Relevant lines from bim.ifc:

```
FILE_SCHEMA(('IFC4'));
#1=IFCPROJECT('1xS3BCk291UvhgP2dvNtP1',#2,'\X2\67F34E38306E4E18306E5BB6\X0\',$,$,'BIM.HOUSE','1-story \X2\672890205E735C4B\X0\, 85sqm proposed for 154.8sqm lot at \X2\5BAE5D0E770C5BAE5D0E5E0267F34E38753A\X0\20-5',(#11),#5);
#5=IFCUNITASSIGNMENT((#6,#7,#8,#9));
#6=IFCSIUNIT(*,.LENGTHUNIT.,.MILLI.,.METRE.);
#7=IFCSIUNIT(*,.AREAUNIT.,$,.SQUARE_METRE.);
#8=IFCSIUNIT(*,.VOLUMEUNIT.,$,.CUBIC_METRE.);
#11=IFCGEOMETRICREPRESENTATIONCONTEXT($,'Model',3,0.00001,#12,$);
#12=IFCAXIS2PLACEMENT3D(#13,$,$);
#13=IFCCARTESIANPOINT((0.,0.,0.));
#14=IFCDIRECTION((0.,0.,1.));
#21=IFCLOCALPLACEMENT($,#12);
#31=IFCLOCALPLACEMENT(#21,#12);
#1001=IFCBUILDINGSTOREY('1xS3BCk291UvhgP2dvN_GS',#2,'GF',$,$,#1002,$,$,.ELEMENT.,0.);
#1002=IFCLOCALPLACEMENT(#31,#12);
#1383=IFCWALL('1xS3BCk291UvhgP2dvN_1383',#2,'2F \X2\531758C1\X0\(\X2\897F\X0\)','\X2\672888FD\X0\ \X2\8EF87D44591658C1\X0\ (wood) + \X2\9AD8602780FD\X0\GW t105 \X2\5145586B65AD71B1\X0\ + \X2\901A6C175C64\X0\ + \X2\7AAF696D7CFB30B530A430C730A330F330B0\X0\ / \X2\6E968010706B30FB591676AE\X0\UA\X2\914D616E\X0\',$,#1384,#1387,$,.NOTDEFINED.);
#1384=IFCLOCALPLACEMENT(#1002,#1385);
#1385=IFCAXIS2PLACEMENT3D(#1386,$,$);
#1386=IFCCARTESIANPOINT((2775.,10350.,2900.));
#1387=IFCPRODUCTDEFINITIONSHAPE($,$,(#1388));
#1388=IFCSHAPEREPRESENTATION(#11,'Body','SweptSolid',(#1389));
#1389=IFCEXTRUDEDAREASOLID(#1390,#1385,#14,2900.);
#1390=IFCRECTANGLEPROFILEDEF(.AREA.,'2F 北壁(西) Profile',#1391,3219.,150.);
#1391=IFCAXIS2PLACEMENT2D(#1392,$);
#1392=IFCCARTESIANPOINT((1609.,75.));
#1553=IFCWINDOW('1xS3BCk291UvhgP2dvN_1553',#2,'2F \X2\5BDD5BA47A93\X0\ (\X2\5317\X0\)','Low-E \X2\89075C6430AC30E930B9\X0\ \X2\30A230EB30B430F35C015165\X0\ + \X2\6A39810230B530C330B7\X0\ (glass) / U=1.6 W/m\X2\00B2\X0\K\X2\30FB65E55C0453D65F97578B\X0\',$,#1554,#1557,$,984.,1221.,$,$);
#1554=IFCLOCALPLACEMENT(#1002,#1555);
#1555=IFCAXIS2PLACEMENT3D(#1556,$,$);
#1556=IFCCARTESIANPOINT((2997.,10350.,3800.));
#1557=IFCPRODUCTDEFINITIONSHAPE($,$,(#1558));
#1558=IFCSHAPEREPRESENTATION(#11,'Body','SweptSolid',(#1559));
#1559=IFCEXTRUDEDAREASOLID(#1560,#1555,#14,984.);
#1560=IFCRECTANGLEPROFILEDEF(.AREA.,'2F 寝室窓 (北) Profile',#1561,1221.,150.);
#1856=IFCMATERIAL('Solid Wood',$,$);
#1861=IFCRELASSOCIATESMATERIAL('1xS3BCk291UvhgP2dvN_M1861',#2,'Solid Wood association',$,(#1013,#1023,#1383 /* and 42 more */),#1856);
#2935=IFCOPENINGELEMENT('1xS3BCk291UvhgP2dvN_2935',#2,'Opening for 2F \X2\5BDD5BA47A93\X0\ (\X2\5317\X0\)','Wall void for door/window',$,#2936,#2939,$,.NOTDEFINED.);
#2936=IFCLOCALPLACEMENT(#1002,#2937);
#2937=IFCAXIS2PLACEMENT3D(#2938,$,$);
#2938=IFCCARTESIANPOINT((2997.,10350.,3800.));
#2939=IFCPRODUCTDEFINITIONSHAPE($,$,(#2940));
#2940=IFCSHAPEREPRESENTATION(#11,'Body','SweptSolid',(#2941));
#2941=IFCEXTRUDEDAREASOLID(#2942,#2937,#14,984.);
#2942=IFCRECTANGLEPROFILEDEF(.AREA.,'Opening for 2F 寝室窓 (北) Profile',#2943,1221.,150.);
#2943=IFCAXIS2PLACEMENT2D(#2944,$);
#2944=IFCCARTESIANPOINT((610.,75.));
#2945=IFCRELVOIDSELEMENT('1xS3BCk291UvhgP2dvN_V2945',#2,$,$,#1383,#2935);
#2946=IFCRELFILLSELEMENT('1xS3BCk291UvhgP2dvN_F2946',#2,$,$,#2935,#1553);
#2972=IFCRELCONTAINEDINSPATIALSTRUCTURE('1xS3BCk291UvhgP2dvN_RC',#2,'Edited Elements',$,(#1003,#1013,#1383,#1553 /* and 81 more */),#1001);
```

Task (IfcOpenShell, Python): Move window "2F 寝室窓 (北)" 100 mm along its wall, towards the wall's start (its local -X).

```python
import ifcopenshell
import ifcopenshell.api.geometry
import ifcopenshell.util.placement

model = ifcopenshell.open("bim.ifc")

window = model.by_guid("1xS3BCk291UvhgP2dvN_1553")
opening = window.FillsVoids[0].RelatingOpeningElement
wall = opening.VoidsElements[0].RelatingBuildingElement

wall_matrix = ifcopenshell.util.placement.get_local_placement(wall.ObjectPlacement)
shift = wall_matrix[:3, 0] * -100.0
before = ifcopenshell.util.placement.get_local_placement(window.ObjectPlacement)[:3, 3].copy()

# The window is not placed relative to its opening, so move both.
for product in (opening, window):
    matrix = ifcopenshell.util.placement.get_local_placement(product.ObjectPlacement)
    matrix[:3, 3] += shift
    ifcopenshell.api.geometry.edit_object_placement(model, product=product, matrix=matrix, is_si=False)

after = ifcopenshell.util.placement.get_local_placement(window.ObjectPlacement)[:3, 3]
print("window moved by", (after - before).round(3) + 0.0)

model.write("bim_updated.ifc")
```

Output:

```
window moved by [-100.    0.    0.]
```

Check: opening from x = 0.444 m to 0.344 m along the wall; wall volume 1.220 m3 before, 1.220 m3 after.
